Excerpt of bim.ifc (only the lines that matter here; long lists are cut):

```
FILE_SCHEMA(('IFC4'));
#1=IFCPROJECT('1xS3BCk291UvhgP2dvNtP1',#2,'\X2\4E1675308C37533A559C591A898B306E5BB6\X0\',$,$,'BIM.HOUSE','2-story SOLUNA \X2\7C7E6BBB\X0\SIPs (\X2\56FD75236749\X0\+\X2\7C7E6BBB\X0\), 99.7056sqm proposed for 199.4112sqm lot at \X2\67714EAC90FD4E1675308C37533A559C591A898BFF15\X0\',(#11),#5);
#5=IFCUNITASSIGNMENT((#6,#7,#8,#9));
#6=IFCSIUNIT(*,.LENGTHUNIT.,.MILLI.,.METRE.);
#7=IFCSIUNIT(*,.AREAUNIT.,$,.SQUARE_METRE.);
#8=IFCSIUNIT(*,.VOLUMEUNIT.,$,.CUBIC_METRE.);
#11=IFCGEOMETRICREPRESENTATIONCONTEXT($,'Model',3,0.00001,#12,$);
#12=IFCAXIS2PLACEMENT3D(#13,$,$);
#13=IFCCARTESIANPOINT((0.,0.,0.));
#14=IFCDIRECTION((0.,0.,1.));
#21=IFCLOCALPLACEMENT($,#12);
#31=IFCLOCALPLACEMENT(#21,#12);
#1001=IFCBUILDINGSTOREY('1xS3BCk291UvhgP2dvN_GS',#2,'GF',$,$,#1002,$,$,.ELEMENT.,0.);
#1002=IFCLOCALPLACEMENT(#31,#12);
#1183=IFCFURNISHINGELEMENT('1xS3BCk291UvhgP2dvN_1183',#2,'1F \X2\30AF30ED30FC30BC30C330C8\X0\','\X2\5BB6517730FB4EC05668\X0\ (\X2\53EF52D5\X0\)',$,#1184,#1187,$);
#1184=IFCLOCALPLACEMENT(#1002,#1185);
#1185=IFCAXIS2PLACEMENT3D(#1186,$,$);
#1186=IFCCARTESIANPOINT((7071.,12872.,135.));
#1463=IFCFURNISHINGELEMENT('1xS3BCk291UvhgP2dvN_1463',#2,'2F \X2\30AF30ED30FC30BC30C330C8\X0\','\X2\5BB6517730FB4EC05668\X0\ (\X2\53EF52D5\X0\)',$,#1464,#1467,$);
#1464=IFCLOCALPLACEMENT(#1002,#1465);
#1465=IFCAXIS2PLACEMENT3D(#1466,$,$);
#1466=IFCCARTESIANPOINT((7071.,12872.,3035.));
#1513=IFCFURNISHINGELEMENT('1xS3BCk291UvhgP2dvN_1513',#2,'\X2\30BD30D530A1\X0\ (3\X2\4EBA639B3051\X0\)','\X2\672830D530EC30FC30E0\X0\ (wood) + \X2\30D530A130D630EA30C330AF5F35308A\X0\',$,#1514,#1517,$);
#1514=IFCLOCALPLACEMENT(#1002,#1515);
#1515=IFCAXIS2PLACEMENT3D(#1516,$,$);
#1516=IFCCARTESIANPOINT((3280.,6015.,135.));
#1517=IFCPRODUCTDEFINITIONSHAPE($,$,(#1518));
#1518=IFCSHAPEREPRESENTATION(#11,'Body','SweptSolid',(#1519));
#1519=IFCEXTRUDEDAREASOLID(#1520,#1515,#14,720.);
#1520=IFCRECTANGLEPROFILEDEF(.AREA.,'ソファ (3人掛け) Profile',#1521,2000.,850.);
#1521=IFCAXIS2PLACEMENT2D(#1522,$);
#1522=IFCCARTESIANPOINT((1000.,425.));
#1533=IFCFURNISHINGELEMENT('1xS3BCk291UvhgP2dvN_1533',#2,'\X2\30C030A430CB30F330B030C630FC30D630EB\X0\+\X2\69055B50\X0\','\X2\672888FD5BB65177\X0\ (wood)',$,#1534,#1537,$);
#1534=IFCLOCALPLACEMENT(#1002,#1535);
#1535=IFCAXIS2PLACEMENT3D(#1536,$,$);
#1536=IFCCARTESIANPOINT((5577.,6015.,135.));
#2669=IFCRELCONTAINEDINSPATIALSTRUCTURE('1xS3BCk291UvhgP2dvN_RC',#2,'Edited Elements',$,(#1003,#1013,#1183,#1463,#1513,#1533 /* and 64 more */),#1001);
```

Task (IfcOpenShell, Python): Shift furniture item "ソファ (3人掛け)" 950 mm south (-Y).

```python
import ifcopenshell
import ifcopenshell.api.geometry
import ifcopenshell.util.placement

model = ifcopenshell.open("bim.ifc")

item = model.by_guid("1xS3BCk291UvhgP2dvN_1513")
matrix = ifcopenshell.util.placement.get_local_placement(item.ObjectPlacement)
matrix[1, 3] -= 950.0
ifcopenshell.api.geometry.edit_object_placement(model, product=item, matrix=matrix, is_si=False)

print(ifcopenshell.util.placement.get_local_placement(item.ObjectPlacement).round(3) + 0.0)

model.write("bim_edited.ifc")
```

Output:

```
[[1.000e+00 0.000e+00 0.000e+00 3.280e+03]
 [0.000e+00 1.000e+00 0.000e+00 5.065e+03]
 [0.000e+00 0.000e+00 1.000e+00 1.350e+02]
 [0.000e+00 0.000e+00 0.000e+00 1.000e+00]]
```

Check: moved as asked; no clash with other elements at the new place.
